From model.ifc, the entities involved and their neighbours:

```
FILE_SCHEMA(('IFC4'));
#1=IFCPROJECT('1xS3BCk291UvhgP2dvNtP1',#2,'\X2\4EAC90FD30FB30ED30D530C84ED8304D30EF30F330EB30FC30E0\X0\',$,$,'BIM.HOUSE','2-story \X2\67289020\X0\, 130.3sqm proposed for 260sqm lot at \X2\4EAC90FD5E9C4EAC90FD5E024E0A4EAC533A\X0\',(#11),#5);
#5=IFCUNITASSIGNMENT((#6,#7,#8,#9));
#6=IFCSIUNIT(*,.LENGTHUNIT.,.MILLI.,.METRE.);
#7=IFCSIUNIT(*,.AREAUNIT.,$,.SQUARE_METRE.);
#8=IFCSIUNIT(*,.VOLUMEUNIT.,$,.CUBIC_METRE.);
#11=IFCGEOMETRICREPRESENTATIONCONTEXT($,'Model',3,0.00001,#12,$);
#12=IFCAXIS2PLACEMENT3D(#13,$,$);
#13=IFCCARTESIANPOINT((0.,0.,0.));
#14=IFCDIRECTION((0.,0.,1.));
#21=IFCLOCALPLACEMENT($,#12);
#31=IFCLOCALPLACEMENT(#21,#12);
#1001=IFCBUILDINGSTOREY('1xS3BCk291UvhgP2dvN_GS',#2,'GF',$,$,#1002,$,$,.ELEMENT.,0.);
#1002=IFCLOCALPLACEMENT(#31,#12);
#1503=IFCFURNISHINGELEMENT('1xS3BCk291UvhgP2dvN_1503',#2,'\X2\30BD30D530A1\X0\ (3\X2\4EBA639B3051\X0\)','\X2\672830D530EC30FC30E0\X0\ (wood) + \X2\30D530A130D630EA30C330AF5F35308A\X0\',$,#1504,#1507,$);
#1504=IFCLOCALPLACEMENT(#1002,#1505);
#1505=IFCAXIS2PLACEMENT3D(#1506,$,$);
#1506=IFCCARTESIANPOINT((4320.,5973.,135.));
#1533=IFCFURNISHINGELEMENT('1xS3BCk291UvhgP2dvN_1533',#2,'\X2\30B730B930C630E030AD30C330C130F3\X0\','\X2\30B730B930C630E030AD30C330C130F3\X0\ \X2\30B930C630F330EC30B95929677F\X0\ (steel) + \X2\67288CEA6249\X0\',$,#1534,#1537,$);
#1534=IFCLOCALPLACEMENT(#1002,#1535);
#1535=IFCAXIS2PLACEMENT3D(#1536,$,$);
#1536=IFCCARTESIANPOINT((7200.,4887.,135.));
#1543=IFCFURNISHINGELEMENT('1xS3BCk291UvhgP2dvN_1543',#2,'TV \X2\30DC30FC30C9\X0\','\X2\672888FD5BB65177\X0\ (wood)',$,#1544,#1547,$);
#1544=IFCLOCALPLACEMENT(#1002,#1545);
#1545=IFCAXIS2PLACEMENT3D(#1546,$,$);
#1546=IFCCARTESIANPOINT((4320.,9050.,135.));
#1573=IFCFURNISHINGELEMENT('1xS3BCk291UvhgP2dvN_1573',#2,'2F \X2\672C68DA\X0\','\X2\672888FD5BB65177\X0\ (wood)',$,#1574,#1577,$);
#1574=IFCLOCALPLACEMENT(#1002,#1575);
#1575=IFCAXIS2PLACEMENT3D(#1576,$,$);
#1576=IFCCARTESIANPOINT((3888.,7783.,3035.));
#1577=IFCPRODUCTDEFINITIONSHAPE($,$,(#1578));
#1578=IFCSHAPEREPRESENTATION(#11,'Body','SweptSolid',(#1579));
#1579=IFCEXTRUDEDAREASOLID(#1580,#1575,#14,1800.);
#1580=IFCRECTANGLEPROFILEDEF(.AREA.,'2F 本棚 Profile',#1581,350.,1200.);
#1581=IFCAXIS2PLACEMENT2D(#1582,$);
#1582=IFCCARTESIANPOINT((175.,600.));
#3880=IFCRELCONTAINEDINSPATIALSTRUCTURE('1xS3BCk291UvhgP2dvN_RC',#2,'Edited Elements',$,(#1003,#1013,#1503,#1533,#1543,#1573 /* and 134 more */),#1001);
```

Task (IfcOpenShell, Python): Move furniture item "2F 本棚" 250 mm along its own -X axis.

```python
import ifcopenshell
import ifcopenshell.api.geometry
import ifcopenshell.util.placement

model = ifcopenshell.open("model.ifc")

item = model.by_guid("1xS3BCk291UvhgP2dvN_1573")
matrix = ifcopenshell.util.placement.get_local_placement(item.ObjectPlacement)
matrix[:3, 3] -= matrix[:3, 0] * 250.0
ifcopenshell.api.geometry.edit_object_placement(model, product=item, matrix=matrix, is_si=False)

print(ifcopenshell.util.placement.get_local_placement(item.ObjectPlacement).round(3) + 0.0)

model.write("model_rev.ifc")
```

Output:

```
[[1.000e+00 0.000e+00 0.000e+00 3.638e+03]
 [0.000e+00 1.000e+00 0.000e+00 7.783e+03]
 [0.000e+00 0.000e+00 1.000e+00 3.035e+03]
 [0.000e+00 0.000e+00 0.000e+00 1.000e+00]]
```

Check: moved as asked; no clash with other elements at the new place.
